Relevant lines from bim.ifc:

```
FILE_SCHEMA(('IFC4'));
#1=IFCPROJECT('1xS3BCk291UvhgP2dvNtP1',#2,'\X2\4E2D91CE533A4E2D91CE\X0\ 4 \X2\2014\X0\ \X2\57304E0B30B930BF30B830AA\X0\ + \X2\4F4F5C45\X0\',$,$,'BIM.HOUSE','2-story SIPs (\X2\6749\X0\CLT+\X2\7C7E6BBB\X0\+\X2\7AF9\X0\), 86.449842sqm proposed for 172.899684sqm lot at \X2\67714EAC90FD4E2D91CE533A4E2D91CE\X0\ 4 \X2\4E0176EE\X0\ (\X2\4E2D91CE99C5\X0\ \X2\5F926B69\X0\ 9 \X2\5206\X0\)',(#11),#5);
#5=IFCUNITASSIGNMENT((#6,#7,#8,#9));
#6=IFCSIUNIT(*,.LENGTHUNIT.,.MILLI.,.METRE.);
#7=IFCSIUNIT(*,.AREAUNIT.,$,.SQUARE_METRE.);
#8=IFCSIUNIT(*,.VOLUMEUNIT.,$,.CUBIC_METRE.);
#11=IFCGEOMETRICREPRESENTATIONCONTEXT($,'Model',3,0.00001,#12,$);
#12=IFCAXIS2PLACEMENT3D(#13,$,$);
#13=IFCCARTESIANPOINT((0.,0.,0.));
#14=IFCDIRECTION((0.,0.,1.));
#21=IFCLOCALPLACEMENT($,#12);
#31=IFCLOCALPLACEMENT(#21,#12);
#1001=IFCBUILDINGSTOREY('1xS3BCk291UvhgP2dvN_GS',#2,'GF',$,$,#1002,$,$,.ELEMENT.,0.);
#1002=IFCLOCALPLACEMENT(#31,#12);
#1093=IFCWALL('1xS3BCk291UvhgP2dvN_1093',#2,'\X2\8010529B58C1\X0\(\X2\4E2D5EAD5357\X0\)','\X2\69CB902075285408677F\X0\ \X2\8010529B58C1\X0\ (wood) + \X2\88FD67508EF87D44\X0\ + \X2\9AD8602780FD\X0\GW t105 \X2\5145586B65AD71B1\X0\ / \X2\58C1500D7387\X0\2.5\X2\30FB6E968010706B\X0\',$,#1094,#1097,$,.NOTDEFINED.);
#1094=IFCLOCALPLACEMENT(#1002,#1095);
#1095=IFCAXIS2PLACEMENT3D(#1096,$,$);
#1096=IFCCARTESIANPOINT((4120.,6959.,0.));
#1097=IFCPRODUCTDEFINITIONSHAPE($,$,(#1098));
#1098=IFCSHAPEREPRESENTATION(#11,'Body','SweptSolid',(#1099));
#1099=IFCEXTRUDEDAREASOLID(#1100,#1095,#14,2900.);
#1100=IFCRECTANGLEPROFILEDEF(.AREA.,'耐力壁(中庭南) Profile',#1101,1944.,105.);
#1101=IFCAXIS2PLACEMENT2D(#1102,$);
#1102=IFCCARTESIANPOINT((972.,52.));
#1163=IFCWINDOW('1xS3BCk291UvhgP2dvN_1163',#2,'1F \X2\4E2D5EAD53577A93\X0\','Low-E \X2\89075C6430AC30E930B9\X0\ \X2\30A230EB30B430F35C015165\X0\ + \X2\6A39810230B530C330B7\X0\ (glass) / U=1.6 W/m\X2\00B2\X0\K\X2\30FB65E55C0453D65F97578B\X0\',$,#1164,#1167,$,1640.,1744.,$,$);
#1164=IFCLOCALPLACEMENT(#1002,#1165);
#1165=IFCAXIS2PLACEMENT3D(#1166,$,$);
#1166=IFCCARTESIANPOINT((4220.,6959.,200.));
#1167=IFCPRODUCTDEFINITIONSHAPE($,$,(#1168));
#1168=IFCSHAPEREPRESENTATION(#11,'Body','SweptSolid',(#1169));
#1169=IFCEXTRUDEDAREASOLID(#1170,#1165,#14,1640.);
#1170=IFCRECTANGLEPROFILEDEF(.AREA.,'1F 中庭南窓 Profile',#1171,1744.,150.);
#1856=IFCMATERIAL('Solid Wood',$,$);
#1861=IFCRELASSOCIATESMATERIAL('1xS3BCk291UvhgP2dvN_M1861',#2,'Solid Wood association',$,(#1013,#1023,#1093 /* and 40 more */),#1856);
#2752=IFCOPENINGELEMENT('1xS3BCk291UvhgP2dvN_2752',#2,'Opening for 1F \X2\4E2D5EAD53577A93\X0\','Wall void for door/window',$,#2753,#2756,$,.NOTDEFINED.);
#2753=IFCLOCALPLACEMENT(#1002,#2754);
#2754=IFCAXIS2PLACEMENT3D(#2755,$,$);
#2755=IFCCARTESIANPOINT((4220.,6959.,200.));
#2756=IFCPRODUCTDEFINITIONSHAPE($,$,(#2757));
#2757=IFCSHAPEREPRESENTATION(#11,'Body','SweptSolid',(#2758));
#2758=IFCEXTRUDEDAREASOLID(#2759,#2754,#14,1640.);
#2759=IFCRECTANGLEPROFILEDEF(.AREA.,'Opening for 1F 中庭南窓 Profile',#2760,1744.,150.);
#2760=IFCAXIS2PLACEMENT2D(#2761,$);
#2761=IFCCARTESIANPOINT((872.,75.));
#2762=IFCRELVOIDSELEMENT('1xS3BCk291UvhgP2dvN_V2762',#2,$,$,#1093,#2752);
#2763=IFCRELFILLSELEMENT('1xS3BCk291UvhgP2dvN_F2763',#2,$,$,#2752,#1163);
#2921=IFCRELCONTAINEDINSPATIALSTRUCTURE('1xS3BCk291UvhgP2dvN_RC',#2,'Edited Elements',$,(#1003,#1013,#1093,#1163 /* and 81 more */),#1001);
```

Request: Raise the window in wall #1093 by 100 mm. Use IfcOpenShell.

```python
import numpy as np
import ifcopenshell
import ifcopenshell.api.geometry
import ifcopenshell.util.placement
import ifcopenshell.util.unit

model = ifcopenshell.open("bim.ifc")
unit_scale = ifcopenshell.util.unit.calculate_unit_scale(model)

window = model.by_id(1163)
opening = window.FillsVoids[0].RelatingOpeningElement
dz = 100.0

shift = np.array([0.0, 0.0, dz])
# The window is not placed relative to its opening, so move both.
for product in (opening, window):
    matrix = ifcopenshell.util.placement.get_local_placement(product.ObjectPlacement)
    matrix[:3, 3] += shift
    ifcopenshell.api.geometry.edit_object_placement(model, product=product, matrix=matrix, is_si=False)

print(f"moved by {dz * unit_scale:+.3f} m")

model.write("bim-out.ifc")
```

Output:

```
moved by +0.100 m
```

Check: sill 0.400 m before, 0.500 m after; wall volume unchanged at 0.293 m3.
